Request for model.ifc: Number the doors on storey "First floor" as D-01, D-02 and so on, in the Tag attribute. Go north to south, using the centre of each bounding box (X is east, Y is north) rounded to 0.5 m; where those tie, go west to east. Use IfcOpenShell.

First a look at what the model holds.

```python
import ifcopenshell
import ifcopenshell.util.element
import ifcopenshell.util.placement

model = ifcopenshell.open("model.ifc")
print(model.schema)
storey = next(s for s in model.by_type("IfcBuildingStorey") if s.Name == "First floor")
doors = [e for e in ifcopenshell.util.element.get_decomposition(storey) if e.is_a("IfcDoor")]
for e in sorted(doors, key=lambda e: e.id()):
    origin = ifcopenshell.util.placement.get_local_placement(e.ObjectPlacement)[:3, 3]
    print(e.id(), e.Tag, e.Name, origin.round(2) + 0.0, sep=" | ")
```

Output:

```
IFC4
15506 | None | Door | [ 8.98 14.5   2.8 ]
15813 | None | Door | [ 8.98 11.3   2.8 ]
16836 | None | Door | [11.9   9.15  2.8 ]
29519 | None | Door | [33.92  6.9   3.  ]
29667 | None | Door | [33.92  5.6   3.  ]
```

```python
import ifcopenshell
import ifcopenshell.geom
import ifcopenshell.util.element
import ifcopenshell.util.shape

model = ifcopenshell.open("model.ifc")
settings = ifcopenshell.geom.settings()
settings.set("use-world-coords", True)


def centre(element):
    shape = ifcopenshell.geom.create_shape(settings, element)
    return ifcopenshell.util.shape.get_bbox_centroid(shape.geometry)


storey = next(s for s in model.by_type("IfcBuildingStorey") if s.Name == "First floor")
doors = [e for e in ifcopenshell.util.element.get_decomposition(storey) if e.is_a("IfcDoor")]

# Insertion points can sit at a corner or the storey origin, so sort by the geometry (in metres).
centres = {e: centre(e) for e in doors}
doors.sort(key=lambda e: (-round(centres[e][1] / 0.5), centres[e][0]))

for i, e in enumerate(doors, start=1):
    number = f"D-{i:02d}"
    e.Tag = number
    print(e.id(), number)

model.write("model_rev.ifc")
```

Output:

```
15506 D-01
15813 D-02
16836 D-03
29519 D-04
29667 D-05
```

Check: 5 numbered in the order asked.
